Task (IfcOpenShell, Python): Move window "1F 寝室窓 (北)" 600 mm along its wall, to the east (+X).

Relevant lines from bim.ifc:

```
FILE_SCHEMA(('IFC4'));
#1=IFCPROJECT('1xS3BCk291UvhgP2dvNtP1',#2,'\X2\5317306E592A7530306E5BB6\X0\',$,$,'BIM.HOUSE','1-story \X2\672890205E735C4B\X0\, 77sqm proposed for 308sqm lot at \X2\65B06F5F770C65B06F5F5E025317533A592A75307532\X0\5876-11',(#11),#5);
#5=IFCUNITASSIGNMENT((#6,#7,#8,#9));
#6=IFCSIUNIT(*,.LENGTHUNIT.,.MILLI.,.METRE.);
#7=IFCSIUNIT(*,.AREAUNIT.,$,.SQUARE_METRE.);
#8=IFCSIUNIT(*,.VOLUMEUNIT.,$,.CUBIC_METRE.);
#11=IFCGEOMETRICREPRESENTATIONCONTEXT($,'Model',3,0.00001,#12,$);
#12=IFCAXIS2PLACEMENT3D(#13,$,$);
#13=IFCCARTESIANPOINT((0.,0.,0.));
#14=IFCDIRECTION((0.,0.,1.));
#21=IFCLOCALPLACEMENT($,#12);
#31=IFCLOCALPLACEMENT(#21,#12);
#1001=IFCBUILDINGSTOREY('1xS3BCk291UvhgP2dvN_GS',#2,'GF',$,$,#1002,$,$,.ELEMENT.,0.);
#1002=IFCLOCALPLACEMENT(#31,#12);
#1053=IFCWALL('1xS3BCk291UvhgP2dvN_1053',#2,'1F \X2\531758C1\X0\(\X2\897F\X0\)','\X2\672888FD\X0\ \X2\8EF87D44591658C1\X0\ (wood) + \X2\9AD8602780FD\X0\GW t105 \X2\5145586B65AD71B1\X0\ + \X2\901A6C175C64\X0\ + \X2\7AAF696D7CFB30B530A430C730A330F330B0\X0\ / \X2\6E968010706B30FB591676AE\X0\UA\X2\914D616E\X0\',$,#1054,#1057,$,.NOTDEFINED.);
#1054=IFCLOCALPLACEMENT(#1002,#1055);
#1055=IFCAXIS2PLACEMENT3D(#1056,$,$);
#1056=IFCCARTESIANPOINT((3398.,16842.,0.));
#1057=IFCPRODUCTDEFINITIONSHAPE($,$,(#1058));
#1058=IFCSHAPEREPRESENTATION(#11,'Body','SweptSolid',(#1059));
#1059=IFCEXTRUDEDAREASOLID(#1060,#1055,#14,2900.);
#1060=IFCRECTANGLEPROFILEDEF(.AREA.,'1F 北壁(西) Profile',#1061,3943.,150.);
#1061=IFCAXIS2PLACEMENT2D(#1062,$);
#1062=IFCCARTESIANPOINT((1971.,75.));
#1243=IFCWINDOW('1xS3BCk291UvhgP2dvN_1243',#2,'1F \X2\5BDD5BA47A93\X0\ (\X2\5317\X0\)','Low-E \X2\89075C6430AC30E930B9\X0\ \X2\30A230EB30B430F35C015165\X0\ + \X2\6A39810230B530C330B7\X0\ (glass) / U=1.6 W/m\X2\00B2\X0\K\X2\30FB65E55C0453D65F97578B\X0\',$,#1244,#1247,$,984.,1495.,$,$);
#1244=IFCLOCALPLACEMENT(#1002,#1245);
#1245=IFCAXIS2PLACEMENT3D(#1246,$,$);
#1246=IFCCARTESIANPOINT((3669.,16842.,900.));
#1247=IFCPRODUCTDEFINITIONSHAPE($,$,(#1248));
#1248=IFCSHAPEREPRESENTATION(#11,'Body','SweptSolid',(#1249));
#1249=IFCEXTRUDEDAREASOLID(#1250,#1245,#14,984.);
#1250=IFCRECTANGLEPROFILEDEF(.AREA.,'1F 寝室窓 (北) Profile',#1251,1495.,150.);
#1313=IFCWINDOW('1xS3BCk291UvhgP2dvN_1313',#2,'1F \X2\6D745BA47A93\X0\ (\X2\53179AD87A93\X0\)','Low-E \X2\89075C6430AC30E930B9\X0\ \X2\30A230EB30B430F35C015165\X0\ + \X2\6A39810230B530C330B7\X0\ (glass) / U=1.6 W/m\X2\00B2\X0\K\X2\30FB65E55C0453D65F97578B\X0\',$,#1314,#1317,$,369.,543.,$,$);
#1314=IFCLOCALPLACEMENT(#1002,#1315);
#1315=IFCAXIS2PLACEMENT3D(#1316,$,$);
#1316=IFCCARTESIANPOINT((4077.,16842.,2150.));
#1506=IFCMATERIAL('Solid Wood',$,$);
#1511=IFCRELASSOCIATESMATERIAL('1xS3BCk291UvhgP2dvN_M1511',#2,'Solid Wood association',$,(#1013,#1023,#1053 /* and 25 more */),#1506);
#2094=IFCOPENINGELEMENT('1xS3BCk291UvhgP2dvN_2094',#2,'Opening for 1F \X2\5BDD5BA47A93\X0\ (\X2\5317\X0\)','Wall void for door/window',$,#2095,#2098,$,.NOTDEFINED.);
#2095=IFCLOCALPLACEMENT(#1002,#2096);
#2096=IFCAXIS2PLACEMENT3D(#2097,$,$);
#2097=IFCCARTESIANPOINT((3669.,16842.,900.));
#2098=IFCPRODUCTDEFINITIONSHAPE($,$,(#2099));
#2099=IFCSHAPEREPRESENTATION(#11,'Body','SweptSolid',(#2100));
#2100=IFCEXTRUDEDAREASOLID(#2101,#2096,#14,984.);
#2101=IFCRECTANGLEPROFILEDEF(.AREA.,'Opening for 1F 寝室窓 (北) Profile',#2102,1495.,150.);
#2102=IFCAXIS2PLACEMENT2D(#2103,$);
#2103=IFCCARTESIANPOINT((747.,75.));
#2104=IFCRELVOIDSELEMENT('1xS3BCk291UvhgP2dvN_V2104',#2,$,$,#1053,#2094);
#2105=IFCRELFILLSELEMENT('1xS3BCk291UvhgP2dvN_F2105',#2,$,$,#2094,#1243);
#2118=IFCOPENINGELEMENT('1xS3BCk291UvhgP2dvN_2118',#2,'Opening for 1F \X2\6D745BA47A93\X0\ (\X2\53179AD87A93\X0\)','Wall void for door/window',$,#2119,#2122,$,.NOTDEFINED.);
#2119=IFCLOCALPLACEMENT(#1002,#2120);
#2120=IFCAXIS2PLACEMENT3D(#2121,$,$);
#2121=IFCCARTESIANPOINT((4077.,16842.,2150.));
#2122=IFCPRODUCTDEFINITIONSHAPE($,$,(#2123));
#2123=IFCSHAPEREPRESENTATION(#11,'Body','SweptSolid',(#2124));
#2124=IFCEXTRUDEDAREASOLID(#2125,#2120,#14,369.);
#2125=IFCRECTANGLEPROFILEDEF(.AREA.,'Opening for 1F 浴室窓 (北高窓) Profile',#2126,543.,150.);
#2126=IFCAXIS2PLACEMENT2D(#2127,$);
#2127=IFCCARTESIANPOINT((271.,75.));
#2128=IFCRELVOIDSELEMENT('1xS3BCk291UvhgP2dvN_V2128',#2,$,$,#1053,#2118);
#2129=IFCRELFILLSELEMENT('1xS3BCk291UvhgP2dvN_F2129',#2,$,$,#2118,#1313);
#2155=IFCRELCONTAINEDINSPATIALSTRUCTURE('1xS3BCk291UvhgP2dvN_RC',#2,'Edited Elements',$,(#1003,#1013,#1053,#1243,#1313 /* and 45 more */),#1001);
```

```python
import ifcopenshell
import ifcopenshell.api.geometry
import ifcopenshell.util.placement
import ifcopenshell.util.unit

model = ifcopenshell.open("bim.ifc")
unit_scale = ifcopenshell.util.unit.calculate_unit_scale(model)

window = model.by_guid("1xS3BCk291UvhgP2dvN_1243")
opening = window.FillsVoids[0].RelatingOpeningElement
wall = opening.VoidsElements[0].RelatingBuildingElement

wall_matrix = ifcopenshell.util.placement.get_local_placement(wall.ObjectPlacement)
shift = wall_matrix[:3, 0] * 0.6 / unit_scale
before = ifcopenshell.util.placement.get_local_placement(window.ObjectPlacement)[:3, 3].copy()

# The window is not placed relative to its opening, so move both.
for product in (opening, window):
    matrix = ifcopenshell.util.placement.get_local_placement(product.ObjectPlacement)
    matrix[:3, 3] += shift
    ifcopenshell.api.geometry.edit_object_placement(model, product=product, matrix=matrix, is_si=False)

after = ifcopenshell.util.placement.get_local_placement(window.ObjectPlacement)[:3, 3]
print("window moved by", (after - before).round(3) + 0.0)

model.write("bim_v2.ifc")
```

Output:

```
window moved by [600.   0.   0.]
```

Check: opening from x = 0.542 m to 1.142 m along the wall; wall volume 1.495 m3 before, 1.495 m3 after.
